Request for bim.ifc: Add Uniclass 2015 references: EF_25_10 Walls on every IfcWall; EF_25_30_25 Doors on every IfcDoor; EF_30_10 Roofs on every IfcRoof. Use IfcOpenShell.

First a look at what the model holds.

```python
import ifcopenshell

model = ifcopenshell.open("bim.ifc")
print(model.schema)
print("classifications:", [c.Name for c in model.by_type("IfcClassification")])
for ifc_class in ("IfcDoor", "IfcRoof", "IfcStair", "IfcWall", "IfcWindow"):
    print(ifc_class, len(model.by_type(ifc_class)))
```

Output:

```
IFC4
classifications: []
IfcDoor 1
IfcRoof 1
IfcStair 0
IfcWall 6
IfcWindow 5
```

```python
import ifcopenshell
import ifcopenshell.api.classification

model = ifcopenshell.open("bim.ifc")

system = ifcopenshell.api.classification.add_classification(model, classification="Uniclass 2015")

codes = {
    "IfcWall": ("EF_25_10", "Walls"),
    "IfcDoor": ("EF_25_30_25", "Doors"),
    "IfcRoof": ("EF_30_10", "Roofs"),
}
for ifc_class, (code, name) in codes.items():
    products = model.by_type(ifc_class)
    ifcopenshell.api.classification.add_reference(
        model, products=products, classification=system, identification=code, name=name
    )
    print(code, len(products))

model.write("bim_edited.ifc")
```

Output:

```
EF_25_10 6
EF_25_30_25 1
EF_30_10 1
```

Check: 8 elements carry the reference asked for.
